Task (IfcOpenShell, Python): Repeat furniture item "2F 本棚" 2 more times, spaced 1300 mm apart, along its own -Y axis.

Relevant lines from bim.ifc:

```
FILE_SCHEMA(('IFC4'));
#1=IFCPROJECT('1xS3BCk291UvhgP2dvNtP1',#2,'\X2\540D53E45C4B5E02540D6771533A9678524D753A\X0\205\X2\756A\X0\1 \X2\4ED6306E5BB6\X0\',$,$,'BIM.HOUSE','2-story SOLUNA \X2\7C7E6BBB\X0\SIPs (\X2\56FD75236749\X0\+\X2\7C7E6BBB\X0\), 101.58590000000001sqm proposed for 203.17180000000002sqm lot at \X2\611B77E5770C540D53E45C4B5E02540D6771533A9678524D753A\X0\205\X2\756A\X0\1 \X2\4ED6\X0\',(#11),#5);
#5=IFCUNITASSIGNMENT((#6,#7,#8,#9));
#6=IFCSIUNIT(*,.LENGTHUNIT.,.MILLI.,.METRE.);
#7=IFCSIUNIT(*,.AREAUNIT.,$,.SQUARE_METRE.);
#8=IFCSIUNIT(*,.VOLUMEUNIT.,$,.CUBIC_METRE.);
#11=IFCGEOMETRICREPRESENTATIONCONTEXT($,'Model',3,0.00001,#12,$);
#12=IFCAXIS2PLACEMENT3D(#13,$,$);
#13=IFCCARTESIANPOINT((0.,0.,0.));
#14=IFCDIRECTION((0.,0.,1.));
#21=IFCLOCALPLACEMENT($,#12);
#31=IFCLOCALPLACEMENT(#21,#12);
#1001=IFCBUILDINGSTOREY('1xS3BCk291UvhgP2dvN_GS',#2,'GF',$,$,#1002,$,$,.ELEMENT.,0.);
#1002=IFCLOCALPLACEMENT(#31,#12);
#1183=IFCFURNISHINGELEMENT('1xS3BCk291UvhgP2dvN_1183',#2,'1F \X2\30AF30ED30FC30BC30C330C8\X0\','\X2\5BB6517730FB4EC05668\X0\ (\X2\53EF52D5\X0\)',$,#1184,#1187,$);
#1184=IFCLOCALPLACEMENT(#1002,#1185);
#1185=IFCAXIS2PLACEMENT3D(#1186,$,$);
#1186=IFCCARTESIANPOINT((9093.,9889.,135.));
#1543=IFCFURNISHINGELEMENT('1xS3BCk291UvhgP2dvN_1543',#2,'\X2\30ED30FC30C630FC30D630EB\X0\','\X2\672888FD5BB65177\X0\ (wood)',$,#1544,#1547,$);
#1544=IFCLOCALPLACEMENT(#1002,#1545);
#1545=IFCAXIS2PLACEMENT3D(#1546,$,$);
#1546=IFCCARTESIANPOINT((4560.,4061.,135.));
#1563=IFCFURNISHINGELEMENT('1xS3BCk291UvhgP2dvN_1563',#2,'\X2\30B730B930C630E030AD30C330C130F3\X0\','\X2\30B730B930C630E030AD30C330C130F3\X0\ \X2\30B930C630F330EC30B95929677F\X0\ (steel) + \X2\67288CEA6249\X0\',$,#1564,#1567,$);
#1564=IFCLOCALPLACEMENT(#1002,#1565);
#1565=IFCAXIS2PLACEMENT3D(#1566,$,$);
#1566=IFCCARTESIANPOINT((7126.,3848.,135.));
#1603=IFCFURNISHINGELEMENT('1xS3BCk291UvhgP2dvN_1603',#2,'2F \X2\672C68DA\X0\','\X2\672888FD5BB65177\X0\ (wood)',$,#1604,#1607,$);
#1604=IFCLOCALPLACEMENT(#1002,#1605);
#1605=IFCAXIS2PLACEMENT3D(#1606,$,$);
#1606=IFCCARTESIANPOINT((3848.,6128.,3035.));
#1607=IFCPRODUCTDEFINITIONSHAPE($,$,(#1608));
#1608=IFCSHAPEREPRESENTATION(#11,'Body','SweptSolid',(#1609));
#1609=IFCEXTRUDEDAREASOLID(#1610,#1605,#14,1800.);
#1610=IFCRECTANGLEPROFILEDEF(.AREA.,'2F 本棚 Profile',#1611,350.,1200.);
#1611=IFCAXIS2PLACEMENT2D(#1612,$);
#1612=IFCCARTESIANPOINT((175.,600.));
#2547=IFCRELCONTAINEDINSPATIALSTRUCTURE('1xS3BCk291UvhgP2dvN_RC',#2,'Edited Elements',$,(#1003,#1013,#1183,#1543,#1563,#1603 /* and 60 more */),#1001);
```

```python
import ifcopenshell
import ifcopenshell.api.geometry
import ifcopenshell.api.root
import ifcopenshell.util.element
import ifcopenshell.util.placement
import ifcopenshell.util.unit

model = ifcopenshell.open("bim.ifc")
unit_scale = ifcopenshell.util.unit.calculate_unit_scale(model)


def reuse_history(source, copy):
    """copy_class also copies each property set's owner history, people and application; keep the originals."""
    for rel in copy.IsDefinedBy:
        if rel.is_a("IfcRelDefinesByProperties") and (history := rel.RelatingPropertyDefinition.OwnerHistory):
            rel.RelatingPropertyDefinition.OwnerHistory = source.OwnerHistory
            ifcopenshell.util.element.remove_deep2(model, history)


source = model.by_guid("1xS3BCk291UvhgP2dvN_1603")
base = ifcopenshell.util.placement.get_local_placement(source.ObjectPlacement)
step = -base[:3, 1] * 1.3 / unit_scale

for i in range(1, 3):
    copy = ifcopenshell.api.root.copy_class(model, product=source)
    copy.Representation = ifcopenshell.util.element.copy_deep(
        model, source.Representation, exclude=["IfcGeometricRepresentationContext", "IfcRepresentationMap"]
    )
    reuse_history(source, copy)
    matrix = base.copy()
    matrix[:3, 3] += i * step
    print("added at", matrix[:3, 3].round(3) + 0.0)
    ifcopenshell.api.geometry.edit_object_placement(model, product=copy, matrix=matrix, is_si=False)

model.write("bim_rev.ifc")
```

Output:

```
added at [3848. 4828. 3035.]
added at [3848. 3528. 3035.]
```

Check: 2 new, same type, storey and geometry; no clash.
